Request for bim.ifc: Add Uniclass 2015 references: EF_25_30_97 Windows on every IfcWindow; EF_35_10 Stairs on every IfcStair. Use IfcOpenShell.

First a look at what the model holds.

```python
import ifcopenshell

model = ifcopenshell.open("bim.ifc")
print(model.schema)
print("classifications:", [c.Name for c in model.by_type("IfcClassification")])
for ifc_class in ("IfcDoor", "IfcRoof", "IfcStair", "IfcWall", "IfcWindow"):
    print(ifc_class, len(model.by_type(ifc_class)))
```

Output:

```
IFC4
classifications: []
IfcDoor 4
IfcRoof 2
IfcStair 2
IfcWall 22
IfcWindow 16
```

```python
import ifcopenshell
import ifcopenshell.api.classification

model = ifcopenshell.open("bim.ifc")

system = ifcopenshell.api.classification.add_classification(model, classification="Uniclass 2015")

codes = {
    "IfcWindow": ("EF_25_30_97", "Windows"),
    "IfcStair": ("EF_35_10", "Stairs"),
}
for ifc_class, (code, name) in codes.items():
    products = model.by_type(ifc_class)
    ifcopenshell.api.classification.add_reference(
        model, products=products, classification=system, identification=code, name=name
    )
    print(code, len(products))

model.write("bim_edited.ifc")
```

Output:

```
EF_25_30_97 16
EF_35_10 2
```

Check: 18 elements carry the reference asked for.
